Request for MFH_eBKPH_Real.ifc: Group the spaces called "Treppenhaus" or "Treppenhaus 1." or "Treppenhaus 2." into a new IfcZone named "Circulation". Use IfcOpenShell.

First a look at what the model holds.

```python
import ifcopenshell

model = ifcopenshell.open("MFH_eBKPH_Real.ifc")
print(model.schema)
seen = {}
for space in model.by_type("IfcSpace"):
    seen[space.LongName] = seen.get(space.LongName, 0) + 1
for name, count in sorted(seen.items(), key=str):
    print(count, "x", name)
print("zones:", [z.Name for z in model.by_type("IfcZone")][:20])
```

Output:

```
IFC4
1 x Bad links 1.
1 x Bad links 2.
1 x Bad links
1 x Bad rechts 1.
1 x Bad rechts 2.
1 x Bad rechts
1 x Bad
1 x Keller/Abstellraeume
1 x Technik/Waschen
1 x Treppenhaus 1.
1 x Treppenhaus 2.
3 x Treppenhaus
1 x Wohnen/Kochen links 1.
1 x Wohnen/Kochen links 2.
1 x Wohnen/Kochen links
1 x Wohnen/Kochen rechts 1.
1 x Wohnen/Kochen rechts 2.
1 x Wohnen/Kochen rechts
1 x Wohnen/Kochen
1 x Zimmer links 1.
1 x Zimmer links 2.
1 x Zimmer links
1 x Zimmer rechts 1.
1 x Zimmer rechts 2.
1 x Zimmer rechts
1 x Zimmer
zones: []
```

```python
import ifcopenshell
import ifcopenshell.api.group
import ifcopenshell.api.root

model = ifcopenshell.open("MFH_eBKPH_Real.ifc")

names = {"Treppenhaus", "Treppenhaus 1.", "Treppenhaus 2."}
spaces = [s for s in model.by_type("IfcSpace") if s.LongName in names]

zone = ifcopenshell.api.root.create_entity(model, ifc_class="IfcZone", name="Circulation")
ifcopenshell.api.group.assign_group(model, products=spaces, group=zone)
print(len(spaces), "spaces in", zone.Name)

model.write("MFH_eBKPH_Real_updated.ifc")
```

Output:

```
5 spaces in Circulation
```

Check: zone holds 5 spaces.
